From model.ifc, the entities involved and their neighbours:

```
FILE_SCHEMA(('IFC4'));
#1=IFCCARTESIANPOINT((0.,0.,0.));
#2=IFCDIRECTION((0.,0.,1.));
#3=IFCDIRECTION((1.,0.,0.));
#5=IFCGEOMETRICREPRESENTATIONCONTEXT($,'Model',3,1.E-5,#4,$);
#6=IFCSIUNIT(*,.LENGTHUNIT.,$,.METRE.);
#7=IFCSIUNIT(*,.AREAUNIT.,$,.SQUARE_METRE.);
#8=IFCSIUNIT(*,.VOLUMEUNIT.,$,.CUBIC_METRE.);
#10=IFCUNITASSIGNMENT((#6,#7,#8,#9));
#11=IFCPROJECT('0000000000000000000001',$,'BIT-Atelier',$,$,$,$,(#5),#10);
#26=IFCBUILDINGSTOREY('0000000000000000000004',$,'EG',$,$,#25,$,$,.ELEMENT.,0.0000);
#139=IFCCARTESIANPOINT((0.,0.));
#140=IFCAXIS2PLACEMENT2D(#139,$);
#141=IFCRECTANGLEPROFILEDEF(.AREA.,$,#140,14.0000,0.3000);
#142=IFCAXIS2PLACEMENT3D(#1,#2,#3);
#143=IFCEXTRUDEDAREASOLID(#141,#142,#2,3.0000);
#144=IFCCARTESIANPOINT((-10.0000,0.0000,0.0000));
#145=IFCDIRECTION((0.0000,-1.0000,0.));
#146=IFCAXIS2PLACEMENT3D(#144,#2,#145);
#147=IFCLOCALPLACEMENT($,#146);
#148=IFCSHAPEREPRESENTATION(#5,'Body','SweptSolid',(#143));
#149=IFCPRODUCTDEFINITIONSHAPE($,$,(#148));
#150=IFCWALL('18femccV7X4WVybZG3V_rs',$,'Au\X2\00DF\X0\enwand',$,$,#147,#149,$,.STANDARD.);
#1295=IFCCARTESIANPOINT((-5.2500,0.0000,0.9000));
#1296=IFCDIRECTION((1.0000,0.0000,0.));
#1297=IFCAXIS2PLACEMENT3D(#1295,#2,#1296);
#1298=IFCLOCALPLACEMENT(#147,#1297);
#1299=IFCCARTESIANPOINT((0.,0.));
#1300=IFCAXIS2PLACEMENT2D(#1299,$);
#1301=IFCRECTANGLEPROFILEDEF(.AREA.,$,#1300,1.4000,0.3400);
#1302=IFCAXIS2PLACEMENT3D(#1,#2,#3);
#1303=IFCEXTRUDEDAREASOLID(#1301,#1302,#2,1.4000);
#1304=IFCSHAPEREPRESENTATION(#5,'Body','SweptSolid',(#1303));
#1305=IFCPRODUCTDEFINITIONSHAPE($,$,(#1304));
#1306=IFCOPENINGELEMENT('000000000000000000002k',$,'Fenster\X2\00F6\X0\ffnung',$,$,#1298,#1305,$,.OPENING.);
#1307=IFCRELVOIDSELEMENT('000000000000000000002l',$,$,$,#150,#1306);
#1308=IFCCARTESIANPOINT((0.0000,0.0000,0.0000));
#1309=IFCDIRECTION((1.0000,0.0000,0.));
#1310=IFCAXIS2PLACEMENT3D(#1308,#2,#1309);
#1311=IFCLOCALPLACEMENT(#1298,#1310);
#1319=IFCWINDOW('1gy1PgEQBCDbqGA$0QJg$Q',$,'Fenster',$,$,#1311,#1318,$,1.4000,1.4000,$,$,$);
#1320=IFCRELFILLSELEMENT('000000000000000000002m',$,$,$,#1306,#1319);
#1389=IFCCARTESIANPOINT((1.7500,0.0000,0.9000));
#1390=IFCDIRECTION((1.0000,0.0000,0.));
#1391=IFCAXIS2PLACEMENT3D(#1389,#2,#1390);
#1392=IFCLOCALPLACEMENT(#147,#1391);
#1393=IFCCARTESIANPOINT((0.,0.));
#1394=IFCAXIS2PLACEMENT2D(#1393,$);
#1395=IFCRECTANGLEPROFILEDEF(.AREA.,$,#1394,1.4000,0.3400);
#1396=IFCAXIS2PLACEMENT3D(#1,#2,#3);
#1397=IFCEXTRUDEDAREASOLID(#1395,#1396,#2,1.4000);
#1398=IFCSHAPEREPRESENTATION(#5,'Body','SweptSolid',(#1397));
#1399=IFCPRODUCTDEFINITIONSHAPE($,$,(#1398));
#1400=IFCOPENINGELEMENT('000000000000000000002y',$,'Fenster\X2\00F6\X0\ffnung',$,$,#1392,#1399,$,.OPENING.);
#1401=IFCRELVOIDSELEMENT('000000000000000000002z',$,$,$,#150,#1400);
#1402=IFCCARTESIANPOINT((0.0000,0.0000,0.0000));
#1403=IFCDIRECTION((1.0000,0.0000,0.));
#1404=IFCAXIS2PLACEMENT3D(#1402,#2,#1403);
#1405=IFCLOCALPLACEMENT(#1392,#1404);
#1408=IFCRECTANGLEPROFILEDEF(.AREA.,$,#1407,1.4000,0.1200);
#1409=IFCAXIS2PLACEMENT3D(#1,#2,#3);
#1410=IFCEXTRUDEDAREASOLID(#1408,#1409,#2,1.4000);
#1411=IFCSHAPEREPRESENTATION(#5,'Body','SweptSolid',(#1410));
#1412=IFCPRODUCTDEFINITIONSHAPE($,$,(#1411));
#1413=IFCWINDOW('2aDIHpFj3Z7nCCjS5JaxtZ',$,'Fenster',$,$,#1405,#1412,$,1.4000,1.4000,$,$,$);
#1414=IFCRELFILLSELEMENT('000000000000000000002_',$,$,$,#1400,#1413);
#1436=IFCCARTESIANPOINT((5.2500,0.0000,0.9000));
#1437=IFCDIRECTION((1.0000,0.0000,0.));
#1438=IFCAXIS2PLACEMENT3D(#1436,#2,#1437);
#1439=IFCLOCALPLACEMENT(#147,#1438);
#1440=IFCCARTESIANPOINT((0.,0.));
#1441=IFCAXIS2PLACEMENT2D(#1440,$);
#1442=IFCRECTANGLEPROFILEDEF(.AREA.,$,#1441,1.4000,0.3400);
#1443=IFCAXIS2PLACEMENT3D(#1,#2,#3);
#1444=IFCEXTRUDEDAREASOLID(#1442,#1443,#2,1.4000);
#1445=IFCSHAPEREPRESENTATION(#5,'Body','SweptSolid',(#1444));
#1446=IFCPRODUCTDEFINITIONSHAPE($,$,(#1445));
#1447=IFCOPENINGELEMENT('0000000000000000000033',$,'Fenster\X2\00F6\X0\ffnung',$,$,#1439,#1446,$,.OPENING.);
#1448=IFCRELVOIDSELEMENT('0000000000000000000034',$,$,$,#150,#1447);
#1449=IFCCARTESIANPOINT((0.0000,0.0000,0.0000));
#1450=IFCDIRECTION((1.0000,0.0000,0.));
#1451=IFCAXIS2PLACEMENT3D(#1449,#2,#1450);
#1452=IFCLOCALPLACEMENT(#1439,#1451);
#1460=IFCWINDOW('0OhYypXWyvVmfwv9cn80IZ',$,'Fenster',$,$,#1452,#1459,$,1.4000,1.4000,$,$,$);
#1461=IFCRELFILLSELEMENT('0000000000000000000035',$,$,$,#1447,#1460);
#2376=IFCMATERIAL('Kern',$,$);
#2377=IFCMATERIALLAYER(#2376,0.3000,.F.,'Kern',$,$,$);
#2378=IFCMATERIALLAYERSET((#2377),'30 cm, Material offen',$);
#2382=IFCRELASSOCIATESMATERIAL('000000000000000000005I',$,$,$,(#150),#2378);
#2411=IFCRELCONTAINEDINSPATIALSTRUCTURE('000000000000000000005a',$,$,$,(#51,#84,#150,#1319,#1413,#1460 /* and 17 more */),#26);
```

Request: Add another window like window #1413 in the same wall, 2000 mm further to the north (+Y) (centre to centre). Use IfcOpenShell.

```python
import ifcopenshell
import ifcopenshell.api.feature
import ifcopenshell.api.geometry
import ifcopenshell.api.root
import ifcopenshell.geom
import ifcopenshell.util.element
import ifcopenshell.util.placement
import ifcopenshell.util.shape
import ifcopenshell.util.unit

model = ifcopenshell.open("model.ifc")
unit_scale = ifcopenshell.util.unit.calculate_unit_scale(model)
settings = ifcopenshell.geom.settings()


def volume(element):
    """Net volume in cubic metres, openings subtracted."""
    shape = ifcopenshell.geom.create_shape(settings, element)
    return ifcopenshell.util.shape.get_volume(shape.geometry)


window = model.by_id(1413)
opening = window.FillsVoids[0].RelatingOpeningElement
wall = opening.VoidsElements[0].RelatingBuildingElement
before = volume(wall)
shift = ifcopenshell.util.placement.get_local_placement(wall.ObjectPlacement)[:3, 0] * -2 / unit_scale

# copy_class copies the void relationship, type, container and properties, but no geometry.
new_opening = ifcopenshell.api.root.copy_class(model, product=opening)
new_opening.Representation = ifcopenshell.util.element.copy_deep(
    model, opening.Representation, exclude=["IfcGeometricRepresentationContext", "IfcRepresentationMap"]
)
new_window = ifcopenshell.api.root.copy_class(model, product=window)
new_window.Representation = ifcopenshell.util.element.copy_deep(
    model, window.Representation, exclude=["IfcGeometricRepresentationContext", "IfcRepresentationMap"]
)
ifcopenshell.api.feature.add_filling(model, opening=new_opening, element=new_window)

for old, new in ((opening, new_opening), (window, new_window)):
    matrix = ifcopenshell.util.placement.get_local_placement(old.ObjectPlacement)
    matrix[:3, 3] += shift
    ifcopenshell.api.geometry.edit_object_placement(model, product=new, matrix=matrix, is_si=False)

after = volume(wall)

print(f"wall volume {before:.3f} -> {after:.3f} m3")

model.write("model_edited.ifc")
```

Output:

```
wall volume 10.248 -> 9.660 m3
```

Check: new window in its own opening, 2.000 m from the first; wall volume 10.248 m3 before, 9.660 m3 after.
